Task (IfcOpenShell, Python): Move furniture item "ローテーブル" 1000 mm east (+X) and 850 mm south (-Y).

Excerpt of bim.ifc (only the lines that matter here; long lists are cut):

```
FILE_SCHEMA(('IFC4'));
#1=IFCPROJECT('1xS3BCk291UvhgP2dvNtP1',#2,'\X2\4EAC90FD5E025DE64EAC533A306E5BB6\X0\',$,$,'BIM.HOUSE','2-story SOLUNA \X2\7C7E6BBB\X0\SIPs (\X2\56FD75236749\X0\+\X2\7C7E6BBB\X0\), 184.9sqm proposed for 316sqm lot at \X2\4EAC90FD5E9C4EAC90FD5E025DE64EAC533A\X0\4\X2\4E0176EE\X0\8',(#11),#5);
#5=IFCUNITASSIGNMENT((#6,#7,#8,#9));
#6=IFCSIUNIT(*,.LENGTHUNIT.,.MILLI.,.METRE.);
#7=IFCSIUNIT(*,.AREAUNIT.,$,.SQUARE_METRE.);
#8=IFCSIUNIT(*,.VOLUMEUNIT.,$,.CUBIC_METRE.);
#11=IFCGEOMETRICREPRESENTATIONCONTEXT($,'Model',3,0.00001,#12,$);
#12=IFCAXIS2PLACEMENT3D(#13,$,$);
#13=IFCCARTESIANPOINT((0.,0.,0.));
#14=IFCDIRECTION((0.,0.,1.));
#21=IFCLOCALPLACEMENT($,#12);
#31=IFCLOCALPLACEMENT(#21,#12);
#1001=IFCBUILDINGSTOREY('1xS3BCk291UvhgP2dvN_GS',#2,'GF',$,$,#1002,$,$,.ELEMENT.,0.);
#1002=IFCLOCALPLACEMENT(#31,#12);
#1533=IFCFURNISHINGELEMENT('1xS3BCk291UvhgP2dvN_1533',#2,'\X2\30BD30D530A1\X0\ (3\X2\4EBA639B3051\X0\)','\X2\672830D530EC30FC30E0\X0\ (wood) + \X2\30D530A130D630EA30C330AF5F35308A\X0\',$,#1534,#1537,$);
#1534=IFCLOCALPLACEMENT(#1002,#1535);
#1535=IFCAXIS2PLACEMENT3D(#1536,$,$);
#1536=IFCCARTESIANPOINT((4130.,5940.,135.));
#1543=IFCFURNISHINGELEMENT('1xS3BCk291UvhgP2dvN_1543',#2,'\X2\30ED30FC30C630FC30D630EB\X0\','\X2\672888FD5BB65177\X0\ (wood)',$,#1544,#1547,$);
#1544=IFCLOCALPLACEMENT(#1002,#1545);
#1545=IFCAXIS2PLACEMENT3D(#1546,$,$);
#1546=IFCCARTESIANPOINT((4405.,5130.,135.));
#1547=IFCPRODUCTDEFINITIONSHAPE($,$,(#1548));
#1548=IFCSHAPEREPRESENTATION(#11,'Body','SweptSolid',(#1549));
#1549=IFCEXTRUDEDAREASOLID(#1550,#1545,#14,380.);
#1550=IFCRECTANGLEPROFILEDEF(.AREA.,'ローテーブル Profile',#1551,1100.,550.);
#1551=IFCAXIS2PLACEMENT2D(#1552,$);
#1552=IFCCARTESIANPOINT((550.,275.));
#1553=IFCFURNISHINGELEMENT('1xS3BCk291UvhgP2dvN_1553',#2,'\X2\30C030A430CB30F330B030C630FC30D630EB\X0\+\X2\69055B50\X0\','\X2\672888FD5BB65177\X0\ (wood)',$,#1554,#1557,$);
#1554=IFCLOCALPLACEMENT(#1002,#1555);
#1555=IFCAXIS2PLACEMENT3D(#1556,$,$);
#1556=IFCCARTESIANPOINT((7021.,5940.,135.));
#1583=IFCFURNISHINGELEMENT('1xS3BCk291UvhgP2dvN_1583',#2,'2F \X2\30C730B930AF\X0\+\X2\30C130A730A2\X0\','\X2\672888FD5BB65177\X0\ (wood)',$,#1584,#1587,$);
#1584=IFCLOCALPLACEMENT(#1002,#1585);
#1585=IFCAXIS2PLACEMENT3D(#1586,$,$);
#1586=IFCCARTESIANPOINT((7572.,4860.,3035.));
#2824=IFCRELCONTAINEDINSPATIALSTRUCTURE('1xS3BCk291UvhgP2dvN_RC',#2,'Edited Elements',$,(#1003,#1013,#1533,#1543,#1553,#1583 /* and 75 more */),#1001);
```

```python
import ifcopenshell
import ifcopenshell.api.geometry
import ifcopenshell.util.placement
import ifcopenshell.util.unit

model = ifcopenshell.open("bim.ifc")
unit_scale = ifcopenshell.util.unit.calculate_unit_scale(model)

item = model.by_guid("1xS3BCk291UvhgP2dvN_1543")
matrix = ifcopenshell.util.placement.get_local_placement(item.ObjectPlacement)
matrix[0, 3] += 1 / unit_scale
matrix[1, 3] -= 0.85 / unit_scale
ifcopenshell.api.geometry.edit_object_placement(model, product=item, matrix=matrix, is_si=False)

print(ifcopenshell.util.placement.get_local_placement(item.ObjectPlacement).round(3) + 0.0)

model.write("bim-out.ifc")
```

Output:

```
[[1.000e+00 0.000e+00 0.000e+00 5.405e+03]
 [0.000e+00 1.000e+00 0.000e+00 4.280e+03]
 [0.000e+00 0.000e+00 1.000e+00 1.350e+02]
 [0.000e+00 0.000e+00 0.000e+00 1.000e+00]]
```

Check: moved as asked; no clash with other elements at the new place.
